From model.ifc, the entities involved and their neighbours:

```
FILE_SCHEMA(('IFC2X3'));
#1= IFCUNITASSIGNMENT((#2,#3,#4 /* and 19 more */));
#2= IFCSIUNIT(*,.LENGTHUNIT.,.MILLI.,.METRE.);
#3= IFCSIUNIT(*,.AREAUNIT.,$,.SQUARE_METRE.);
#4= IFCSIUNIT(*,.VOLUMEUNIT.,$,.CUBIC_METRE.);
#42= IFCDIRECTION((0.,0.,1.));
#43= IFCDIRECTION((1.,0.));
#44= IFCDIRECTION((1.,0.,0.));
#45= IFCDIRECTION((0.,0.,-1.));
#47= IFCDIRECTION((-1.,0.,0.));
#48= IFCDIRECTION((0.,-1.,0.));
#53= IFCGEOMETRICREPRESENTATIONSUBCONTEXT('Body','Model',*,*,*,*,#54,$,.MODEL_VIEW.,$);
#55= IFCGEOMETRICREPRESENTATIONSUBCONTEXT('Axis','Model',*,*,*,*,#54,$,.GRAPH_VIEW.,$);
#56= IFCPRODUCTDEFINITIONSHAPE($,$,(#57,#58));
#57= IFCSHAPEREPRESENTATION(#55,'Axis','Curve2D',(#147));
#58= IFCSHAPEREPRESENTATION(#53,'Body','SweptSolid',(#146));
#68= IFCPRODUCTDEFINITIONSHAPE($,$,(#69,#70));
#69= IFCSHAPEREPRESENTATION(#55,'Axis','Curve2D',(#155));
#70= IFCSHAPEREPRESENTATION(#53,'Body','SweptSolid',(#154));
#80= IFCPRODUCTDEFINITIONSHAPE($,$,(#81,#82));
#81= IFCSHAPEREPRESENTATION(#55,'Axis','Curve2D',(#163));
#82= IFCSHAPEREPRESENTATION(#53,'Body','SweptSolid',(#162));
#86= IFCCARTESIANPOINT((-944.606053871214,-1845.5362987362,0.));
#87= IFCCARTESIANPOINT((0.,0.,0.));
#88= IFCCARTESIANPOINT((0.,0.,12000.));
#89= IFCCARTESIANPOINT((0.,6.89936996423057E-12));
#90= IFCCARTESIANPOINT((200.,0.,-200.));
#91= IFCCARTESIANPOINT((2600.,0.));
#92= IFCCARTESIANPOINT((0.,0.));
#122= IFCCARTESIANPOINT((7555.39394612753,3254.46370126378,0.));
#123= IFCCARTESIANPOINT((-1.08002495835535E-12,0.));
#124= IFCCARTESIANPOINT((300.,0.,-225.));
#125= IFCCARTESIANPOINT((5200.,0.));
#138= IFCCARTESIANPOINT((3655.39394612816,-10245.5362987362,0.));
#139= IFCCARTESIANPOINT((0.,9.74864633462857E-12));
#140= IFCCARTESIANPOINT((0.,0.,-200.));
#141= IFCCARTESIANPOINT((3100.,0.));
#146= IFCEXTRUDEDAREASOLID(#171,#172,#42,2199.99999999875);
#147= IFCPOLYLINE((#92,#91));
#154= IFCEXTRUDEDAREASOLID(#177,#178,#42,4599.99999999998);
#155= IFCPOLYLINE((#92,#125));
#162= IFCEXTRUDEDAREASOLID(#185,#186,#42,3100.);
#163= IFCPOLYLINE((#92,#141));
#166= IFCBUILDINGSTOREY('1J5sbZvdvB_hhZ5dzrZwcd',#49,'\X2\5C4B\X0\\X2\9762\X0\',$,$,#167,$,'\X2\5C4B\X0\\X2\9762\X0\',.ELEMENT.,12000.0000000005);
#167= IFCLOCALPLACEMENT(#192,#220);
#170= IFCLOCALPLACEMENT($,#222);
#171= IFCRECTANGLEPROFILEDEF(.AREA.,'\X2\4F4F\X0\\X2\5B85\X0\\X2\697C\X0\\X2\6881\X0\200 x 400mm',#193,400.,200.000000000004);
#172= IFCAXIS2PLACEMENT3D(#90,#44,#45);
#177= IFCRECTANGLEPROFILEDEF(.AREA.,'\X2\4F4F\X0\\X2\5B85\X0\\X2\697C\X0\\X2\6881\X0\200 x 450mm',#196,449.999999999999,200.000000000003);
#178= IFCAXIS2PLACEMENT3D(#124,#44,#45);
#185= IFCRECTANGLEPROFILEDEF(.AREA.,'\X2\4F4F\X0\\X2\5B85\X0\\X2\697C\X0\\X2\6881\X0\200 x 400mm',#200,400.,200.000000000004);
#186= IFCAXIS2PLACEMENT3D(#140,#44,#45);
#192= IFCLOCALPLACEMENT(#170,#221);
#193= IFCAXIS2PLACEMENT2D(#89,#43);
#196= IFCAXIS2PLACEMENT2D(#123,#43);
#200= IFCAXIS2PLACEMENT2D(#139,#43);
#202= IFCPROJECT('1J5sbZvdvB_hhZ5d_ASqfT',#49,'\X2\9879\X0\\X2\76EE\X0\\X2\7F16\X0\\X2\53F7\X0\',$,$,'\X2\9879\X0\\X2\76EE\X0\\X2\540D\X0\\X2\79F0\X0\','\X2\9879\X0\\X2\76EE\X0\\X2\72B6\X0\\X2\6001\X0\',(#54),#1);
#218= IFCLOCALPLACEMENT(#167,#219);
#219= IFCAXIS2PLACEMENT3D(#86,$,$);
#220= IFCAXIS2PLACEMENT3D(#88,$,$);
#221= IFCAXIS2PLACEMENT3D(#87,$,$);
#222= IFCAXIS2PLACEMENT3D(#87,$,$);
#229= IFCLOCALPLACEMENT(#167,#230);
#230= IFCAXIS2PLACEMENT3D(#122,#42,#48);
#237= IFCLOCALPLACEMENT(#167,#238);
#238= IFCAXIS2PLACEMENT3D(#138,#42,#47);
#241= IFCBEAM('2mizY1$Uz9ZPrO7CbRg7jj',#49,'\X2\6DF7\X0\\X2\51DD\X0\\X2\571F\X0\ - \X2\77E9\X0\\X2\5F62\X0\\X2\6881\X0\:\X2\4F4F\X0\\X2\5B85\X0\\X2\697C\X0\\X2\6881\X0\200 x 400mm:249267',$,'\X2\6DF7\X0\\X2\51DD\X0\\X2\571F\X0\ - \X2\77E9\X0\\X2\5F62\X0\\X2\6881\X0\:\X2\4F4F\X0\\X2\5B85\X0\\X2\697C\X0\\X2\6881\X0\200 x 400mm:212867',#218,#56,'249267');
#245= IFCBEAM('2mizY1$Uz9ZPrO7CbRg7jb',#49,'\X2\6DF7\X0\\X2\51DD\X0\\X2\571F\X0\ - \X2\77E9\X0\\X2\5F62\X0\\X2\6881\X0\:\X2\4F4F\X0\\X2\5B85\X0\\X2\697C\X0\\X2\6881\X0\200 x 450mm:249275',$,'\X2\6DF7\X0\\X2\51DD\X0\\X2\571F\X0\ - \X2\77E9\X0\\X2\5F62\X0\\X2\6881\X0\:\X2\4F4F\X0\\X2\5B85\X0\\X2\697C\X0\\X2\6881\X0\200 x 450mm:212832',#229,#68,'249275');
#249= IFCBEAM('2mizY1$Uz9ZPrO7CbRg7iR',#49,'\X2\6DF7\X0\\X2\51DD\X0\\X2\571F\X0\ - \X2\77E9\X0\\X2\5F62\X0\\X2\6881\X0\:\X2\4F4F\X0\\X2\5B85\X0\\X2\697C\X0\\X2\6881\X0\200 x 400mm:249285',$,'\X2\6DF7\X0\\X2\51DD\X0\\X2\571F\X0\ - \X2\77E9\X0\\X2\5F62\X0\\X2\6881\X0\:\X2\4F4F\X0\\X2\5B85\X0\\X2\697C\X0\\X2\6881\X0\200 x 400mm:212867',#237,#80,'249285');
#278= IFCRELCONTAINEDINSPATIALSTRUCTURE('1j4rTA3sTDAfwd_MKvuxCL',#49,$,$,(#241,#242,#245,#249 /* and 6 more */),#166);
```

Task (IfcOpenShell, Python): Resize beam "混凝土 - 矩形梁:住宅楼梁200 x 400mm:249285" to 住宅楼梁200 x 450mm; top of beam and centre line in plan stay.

```python
import ifcopenshell
import ifcopenshell.util.element
import ifcopenshell.util.representation

model = ifcopenshell.open("model.ifc")

member = model.by_guid("2mizY1$Uz9ZPrO7CbRg7iR")
source = next(p for p in model.by_type("IfcRectangleProfileDef") if p.ProfileName == "住宅楼梁200 x 450mm")

body = ifcopenshell.util.representation.get_representation(member, "Model", "Body")
solid = body.Items[0]
old_profile = solid.SweptArea

# Copy the section's sizes but keep this member's own profile position.
profile = ifcopenshell.util.element.copy(model, source)
# Profiles are centred, so shift by half the change in depth to hold the top.
shift = (old_profile.XDim - profile.XDim) / 2
x, y = old_profile.Position.Location.Coordinates
up = (-1.0, 0.0)  # upwards, in the solid's own plane
location = model.createIfcCartesianPoint((x + up[0] * shift, y + up[1] * shift))
profile.Position = model.createIfcAxis2Placement2D(location, old_profile.Position.RefDirection)
solid.SweptArea = profile
if not model.get_total_inverses(old_profile):
    ifcopenshell.util.element.remove_deep2(model, old_profile)
member.Name = member.Name.replace("住宅楼梁200 x 400mm", "住宅楼梁200 x 450mm")
member.ObjectType = member.ObjectType.replace("住宅楼梁200 x 400mm", "住宅楼梁200 x 450mm")

print(solid.SweptArea)

model.write("model_rev.ifc")
```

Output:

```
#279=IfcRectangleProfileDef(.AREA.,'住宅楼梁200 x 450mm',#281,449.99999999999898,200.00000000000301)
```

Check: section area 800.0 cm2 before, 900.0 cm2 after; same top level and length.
